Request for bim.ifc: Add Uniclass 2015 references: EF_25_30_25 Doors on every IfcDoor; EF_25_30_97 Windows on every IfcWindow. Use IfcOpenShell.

First a look at what the model holds.

```python
import ifcopenshell

model = ifcopenshell.open("bim.ifc")
print(model.schema)
print("classifications:", [c.Name for c in model.by_type("IfcClassification")])
for ifc_class in ("IfcDoor", "IfcRoof", "IfcStair", "IfcWall", "IfcWindow"):
    print(ifc_class, len(model.by_type(ifc_class)))
```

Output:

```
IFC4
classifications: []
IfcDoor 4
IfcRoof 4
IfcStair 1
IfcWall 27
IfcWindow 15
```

```python
import ifcopenshell
import ifcopenshell.api.classification

model = ifcopenshell.open("bim.ifc")

system = ifcopenshell.api.classification.add_classification(model, classification="Uniclass 2015")

codes = {
    "IfcDoor": ("EF_25_30_25", "Doors"),
    "IfcWindow": ("EF_25_30_97", "Windows"),
}
for ifc_class, (code, name) in codes.items():
    products = model.by_type(ifc_class)
    ifcopenshell.api.classification.add_reference(
        model, products=products, classification=system, identification=code, name=name
    )
    print(code, len(products))

model.write("bim_edited.ifc")
```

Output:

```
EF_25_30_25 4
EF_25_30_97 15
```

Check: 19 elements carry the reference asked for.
